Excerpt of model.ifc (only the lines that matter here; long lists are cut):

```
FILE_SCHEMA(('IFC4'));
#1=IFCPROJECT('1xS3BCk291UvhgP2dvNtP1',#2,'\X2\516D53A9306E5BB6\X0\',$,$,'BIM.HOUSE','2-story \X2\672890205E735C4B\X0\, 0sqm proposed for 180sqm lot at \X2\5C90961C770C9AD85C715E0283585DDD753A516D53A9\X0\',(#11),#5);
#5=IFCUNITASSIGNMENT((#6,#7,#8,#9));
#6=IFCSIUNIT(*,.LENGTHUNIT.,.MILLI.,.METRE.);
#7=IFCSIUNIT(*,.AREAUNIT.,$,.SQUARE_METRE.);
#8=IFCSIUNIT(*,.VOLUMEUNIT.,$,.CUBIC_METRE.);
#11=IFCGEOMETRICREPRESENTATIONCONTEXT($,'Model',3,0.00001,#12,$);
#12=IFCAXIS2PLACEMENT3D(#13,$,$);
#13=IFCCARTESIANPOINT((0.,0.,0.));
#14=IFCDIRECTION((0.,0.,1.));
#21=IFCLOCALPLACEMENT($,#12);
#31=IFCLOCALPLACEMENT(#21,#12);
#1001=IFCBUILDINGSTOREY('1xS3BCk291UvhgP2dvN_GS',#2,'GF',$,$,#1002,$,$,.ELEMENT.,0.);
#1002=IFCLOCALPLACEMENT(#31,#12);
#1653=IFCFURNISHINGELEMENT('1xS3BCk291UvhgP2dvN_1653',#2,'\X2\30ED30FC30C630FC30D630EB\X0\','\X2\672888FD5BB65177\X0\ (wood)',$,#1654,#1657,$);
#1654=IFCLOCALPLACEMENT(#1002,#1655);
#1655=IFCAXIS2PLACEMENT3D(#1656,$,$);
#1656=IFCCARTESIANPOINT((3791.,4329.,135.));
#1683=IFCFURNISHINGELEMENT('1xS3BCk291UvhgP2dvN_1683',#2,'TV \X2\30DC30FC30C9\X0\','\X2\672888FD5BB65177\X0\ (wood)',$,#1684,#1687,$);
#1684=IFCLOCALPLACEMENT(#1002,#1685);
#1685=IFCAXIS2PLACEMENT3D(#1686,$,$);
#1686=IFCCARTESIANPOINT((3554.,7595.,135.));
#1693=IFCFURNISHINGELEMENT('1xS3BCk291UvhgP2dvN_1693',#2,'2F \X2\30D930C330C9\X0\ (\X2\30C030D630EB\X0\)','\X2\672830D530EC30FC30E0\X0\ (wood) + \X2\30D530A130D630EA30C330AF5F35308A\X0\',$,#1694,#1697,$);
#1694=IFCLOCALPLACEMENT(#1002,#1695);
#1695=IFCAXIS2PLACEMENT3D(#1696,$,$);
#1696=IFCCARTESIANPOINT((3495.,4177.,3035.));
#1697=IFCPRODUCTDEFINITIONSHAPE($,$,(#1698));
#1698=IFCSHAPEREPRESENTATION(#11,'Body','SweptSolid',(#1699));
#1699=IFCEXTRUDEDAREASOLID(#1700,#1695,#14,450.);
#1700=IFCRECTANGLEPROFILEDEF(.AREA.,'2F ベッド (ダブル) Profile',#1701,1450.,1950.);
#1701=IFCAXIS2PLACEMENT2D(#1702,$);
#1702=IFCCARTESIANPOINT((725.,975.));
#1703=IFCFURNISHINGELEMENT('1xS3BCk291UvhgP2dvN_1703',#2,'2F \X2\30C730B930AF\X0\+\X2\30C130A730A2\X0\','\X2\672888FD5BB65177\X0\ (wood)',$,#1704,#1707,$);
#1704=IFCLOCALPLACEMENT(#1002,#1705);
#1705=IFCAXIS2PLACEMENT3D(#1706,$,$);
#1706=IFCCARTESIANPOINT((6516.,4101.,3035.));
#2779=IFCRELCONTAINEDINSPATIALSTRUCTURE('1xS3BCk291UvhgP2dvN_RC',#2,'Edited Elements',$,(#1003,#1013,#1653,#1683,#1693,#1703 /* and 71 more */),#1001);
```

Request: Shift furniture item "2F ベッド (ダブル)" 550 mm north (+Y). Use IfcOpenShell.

```python
import ifcopenshell
import ifcopenshell.api.geometry
import ifcopenshell.util.placement
import ifcopenshell.util.unit

model = ifcopenshell.open("model.ifc")
unit_scale = ifcopenshell.util.unit.calculate_unit_scale(model)

item = model.by_id(1693)
matrix = ifcopenshell.util.placement.get_local_placement(item.ObjectPlacement)
matrix[1, 3] += 0.55 / unit_scale
ifcopenshell.api.geometry.edit_object_placement(model, product=item, matrix=matrix, is_si=False)

print(ifcopenshell.util.placement.get_local_placement(item.ObjectPlacement).round(3) + 0.0)

model.write("model_edited.ifc")
```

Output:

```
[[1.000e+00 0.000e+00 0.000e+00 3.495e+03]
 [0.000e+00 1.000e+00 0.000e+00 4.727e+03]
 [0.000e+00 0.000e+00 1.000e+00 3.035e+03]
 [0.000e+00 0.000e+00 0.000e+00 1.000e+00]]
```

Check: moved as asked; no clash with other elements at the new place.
